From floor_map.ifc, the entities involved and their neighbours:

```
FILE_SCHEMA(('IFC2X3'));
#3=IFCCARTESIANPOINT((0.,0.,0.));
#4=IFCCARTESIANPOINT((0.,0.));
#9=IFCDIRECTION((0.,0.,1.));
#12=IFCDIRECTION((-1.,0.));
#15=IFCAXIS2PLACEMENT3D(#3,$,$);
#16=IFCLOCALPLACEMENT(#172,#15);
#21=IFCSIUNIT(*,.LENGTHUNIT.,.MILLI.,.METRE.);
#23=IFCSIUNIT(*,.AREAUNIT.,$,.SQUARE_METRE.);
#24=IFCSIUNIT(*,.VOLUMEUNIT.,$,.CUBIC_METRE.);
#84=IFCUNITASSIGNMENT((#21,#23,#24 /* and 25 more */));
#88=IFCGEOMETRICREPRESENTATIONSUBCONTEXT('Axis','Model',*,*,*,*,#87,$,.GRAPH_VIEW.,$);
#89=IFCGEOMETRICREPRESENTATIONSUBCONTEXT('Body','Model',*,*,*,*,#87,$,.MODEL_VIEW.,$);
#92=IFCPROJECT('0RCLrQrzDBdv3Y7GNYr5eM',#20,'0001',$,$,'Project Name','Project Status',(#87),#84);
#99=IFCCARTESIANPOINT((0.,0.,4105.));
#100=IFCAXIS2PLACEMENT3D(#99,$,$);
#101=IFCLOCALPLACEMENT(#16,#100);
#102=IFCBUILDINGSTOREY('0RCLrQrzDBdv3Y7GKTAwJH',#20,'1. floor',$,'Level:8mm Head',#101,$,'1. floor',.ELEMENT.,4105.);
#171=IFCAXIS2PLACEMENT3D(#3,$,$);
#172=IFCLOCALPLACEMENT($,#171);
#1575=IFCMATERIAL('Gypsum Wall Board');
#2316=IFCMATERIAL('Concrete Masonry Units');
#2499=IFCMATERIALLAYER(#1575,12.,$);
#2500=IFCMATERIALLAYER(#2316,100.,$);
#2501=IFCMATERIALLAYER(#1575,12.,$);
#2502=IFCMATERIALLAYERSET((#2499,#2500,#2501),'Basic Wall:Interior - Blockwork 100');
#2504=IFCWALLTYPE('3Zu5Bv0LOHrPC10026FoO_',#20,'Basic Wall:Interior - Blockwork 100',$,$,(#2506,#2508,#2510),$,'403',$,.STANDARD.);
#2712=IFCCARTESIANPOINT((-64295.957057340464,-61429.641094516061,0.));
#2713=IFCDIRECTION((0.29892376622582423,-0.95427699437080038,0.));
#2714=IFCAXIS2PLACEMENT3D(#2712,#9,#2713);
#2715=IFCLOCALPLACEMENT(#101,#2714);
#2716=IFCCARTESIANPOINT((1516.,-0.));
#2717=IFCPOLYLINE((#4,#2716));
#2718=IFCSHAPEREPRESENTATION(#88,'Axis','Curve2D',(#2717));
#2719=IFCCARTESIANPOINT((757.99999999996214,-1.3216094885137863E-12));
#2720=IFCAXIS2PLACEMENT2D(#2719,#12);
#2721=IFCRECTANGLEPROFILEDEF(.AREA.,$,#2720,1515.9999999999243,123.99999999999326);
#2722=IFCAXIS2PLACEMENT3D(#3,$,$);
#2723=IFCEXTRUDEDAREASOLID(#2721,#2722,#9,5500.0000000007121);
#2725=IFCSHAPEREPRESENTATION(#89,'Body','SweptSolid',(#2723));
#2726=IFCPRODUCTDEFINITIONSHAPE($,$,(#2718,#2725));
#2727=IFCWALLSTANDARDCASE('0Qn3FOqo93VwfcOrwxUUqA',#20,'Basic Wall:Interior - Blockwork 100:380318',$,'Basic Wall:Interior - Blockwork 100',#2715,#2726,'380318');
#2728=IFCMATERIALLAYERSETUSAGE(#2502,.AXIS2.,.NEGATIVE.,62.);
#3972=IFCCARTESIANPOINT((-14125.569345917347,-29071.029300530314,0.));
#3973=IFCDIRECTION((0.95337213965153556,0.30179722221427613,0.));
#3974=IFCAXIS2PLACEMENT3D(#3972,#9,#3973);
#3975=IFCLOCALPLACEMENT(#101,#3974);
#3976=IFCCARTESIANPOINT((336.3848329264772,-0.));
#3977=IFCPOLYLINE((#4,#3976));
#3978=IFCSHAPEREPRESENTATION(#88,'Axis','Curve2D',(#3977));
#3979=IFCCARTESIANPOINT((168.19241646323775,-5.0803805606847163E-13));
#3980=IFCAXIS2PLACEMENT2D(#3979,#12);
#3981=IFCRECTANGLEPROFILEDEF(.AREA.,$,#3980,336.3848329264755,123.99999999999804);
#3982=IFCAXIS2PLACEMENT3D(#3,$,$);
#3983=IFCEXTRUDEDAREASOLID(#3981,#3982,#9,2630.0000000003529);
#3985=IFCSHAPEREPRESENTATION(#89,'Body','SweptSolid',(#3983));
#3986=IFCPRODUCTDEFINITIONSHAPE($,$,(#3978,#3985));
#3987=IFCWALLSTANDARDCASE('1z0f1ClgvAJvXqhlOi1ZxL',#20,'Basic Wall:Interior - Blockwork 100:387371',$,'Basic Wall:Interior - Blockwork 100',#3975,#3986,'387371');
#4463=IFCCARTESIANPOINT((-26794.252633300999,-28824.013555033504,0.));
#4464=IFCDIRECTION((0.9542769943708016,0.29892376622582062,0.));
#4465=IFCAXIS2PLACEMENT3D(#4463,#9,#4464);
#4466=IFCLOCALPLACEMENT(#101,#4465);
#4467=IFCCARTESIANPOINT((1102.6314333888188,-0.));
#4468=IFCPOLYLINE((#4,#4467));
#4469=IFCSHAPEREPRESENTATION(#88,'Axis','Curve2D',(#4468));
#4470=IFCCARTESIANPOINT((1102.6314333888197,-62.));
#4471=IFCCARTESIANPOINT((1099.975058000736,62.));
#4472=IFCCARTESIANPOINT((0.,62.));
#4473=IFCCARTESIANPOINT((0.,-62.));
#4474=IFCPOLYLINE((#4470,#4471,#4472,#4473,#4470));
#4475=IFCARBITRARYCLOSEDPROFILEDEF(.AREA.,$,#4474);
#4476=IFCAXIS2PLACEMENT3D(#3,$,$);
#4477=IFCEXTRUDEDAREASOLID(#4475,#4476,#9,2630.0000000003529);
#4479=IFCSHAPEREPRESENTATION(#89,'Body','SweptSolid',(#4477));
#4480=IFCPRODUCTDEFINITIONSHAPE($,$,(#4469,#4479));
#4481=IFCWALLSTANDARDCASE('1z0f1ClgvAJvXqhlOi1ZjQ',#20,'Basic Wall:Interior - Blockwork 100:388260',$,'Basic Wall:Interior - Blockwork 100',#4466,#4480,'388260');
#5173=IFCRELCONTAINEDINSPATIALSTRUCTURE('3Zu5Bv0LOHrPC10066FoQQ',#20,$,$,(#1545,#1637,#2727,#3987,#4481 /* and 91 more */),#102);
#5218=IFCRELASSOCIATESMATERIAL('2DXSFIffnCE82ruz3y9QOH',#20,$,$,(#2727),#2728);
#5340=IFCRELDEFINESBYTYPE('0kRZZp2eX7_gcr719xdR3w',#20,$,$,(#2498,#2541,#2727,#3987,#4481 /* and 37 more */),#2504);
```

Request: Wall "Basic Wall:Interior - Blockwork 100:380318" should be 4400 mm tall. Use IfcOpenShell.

```python
import ifcopenshell
import ifcopenshell.geom
import ifcopenshell.util.representation
import ifcopenshell.util.shape
import ifcopenshell.util.unit

model = ifcopenshell.open("floor_map.ifc")
unit_scale = ifcopenshell.util.unit.calculate_unit_scale(model)
settings = ifcopenshell.geom.settings()


def volume(element):
    """Net volume in cubic metres, openings subtracted."""
    shape = ifcopenshell.geom.create_shape(settings, element)
    return ifcopenshell.util.shape.get_volume(shape.geometry)


wall = model.by_guid("0Qn3FOqo93VwfcOrwxUUqA")
before = volume(wall)

body = ifcopenshell.util.representation.get_representation(wall, "Model", "Body")
solid = body.Items[0]
old_height = solid.Depth
solid.Depth = 4.4 / unit_scale
after = volume(wall)

print(f"height {old_height:g} -> {solid.Depth:g}, volume {before:.3f} -> {after:.3f} m3")

model.write("floor_map_rev.ifc")
```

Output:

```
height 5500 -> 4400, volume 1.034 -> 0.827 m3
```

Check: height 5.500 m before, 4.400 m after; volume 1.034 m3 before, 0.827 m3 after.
